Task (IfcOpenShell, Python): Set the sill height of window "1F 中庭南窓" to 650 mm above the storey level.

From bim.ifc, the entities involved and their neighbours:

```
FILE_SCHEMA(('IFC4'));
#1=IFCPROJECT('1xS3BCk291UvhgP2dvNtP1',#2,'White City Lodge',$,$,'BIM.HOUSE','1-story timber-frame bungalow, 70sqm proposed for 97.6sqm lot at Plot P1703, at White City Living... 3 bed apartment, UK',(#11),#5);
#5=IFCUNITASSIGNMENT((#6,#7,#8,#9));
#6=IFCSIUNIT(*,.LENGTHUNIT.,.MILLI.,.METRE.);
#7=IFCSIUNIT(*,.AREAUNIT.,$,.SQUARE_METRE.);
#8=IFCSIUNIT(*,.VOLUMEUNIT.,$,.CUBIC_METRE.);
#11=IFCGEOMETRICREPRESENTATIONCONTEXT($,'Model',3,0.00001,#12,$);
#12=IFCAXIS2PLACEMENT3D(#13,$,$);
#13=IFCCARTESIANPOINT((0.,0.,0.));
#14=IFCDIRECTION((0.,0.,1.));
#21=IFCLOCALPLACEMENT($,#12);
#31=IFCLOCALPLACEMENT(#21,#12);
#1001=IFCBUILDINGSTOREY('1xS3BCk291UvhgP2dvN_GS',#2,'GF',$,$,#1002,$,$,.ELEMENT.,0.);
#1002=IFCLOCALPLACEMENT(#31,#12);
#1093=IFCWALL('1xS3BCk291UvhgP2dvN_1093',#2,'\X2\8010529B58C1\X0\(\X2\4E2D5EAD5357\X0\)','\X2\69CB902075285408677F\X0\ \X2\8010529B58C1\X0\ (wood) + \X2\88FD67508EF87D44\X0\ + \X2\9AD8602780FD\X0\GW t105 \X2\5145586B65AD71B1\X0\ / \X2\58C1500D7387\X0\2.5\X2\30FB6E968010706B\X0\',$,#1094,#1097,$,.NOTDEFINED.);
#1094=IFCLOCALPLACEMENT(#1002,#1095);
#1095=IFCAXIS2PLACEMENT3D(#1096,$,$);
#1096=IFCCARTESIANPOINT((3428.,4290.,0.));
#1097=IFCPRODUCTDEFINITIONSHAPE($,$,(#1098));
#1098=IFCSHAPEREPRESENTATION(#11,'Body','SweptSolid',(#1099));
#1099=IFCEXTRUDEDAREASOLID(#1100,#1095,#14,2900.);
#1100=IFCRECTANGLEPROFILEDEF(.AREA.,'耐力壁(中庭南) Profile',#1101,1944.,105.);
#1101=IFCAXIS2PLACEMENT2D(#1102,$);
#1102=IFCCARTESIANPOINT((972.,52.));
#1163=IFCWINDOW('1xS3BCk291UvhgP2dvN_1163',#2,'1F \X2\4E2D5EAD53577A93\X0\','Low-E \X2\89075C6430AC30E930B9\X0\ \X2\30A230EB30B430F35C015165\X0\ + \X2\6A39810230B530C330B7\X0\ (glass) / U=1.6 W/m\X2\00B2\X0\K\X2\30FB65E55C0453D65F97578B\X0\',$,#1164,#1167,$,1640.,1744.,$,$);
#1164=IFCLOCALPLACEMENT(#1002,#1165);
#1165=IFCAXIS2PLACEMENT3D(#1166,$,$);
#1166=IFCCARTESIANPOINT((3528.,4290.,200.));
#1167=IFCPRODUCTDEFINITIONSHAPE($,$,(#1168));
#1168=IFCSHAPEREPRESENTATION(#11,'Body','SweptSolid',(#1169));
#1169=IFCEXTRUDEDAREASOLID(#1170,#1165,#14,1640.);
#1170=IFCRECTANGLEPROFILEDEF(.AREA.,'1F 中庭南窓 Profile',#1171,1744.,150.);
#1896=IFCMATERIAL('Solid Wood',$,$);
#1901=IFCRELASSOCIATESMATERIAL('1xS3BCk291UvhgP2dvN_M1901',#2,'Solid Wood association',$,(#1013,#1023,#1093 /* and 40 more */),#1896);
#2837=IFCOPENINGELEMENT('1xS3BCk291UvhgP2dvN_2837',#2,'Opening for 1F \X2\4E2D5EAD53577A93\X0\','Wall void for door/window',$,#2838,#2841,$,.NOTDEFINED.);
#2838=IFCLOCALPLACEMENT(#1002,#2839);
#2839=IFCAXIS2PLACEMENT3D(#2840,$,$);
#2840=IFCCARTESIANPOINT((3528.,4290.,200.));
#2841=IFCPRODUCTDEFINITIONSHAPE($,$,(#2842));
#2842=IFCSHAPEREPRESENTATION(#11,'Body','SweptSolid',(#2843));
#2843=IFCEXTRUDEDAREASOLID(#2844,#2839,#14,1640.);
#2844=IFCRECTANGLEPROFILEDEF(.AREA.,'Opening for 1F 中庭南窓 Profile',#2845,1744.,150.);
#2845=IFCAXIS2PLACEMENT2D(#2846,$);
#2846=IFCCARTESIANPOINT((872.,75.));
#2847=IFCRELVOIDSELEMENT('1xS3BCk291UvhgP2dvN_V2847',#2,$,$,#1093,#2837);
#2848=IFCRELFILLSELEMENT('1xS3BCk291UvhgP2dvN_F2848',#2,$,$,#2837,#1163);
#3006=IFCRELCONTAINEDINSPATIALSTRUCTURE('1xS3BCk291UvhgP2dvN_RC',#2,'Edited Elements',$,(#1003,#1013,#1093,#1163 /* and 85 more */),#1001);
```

```python
import numpy as np
import ifcopenshell
import ifcopenshell.api.geometry
import ifcopenshell.geom
import ifcopenshell.util.element
import ifcopenshell.util.placement
import ifcopenshell.util.shape
import ifcopenshell.util.unit

model = ifcopenshell.open("bim.ifc")
unit_scale = ifcopenshell.util.unit.calculate_unit_scale(model)

window = model.by_id(1163)
opening = window.FillsVoids[0].RelatingOpeningElement
storey = ifcopenshell.util.element.get_container(window, ifc_class="IfcBuildingStorey")
level = ifcopenshell.util.placement.get_local_placement(storey.ObjectPlacement)[2, 3]

# The opening's origin need not be at the sill, so measure its lowest point.
shape = ifcopenshell.geom.create_shape(ifcopenshell.geom.settings(), opening)
bottom = ifcopenshell.util.shape.get_shape_bottom_elevation(shape, shape.geometry) / unit_scale
dz = level + 0.65 / unit_scale - bottom

shift = np.array([0.0, 0.0, dz])
# The window is not placed relative to its opening, so move both.
for product in (opening, window):
    matrix = ifcopenshell.util.placement.get_local_placement(product.ObjectPlacement)
    matrix[:3, 3] += shift
    ifcopenshell.api.geometry.edit_object_placement(model, product=product, matrix=matrix, is_si=False)

print(f"moved by {dz * unit_scale:+.3f} m")

model.write("bim-out.ifc")
```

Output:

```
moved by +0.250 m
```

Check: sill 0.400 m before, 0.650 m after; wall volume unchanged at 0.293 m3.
